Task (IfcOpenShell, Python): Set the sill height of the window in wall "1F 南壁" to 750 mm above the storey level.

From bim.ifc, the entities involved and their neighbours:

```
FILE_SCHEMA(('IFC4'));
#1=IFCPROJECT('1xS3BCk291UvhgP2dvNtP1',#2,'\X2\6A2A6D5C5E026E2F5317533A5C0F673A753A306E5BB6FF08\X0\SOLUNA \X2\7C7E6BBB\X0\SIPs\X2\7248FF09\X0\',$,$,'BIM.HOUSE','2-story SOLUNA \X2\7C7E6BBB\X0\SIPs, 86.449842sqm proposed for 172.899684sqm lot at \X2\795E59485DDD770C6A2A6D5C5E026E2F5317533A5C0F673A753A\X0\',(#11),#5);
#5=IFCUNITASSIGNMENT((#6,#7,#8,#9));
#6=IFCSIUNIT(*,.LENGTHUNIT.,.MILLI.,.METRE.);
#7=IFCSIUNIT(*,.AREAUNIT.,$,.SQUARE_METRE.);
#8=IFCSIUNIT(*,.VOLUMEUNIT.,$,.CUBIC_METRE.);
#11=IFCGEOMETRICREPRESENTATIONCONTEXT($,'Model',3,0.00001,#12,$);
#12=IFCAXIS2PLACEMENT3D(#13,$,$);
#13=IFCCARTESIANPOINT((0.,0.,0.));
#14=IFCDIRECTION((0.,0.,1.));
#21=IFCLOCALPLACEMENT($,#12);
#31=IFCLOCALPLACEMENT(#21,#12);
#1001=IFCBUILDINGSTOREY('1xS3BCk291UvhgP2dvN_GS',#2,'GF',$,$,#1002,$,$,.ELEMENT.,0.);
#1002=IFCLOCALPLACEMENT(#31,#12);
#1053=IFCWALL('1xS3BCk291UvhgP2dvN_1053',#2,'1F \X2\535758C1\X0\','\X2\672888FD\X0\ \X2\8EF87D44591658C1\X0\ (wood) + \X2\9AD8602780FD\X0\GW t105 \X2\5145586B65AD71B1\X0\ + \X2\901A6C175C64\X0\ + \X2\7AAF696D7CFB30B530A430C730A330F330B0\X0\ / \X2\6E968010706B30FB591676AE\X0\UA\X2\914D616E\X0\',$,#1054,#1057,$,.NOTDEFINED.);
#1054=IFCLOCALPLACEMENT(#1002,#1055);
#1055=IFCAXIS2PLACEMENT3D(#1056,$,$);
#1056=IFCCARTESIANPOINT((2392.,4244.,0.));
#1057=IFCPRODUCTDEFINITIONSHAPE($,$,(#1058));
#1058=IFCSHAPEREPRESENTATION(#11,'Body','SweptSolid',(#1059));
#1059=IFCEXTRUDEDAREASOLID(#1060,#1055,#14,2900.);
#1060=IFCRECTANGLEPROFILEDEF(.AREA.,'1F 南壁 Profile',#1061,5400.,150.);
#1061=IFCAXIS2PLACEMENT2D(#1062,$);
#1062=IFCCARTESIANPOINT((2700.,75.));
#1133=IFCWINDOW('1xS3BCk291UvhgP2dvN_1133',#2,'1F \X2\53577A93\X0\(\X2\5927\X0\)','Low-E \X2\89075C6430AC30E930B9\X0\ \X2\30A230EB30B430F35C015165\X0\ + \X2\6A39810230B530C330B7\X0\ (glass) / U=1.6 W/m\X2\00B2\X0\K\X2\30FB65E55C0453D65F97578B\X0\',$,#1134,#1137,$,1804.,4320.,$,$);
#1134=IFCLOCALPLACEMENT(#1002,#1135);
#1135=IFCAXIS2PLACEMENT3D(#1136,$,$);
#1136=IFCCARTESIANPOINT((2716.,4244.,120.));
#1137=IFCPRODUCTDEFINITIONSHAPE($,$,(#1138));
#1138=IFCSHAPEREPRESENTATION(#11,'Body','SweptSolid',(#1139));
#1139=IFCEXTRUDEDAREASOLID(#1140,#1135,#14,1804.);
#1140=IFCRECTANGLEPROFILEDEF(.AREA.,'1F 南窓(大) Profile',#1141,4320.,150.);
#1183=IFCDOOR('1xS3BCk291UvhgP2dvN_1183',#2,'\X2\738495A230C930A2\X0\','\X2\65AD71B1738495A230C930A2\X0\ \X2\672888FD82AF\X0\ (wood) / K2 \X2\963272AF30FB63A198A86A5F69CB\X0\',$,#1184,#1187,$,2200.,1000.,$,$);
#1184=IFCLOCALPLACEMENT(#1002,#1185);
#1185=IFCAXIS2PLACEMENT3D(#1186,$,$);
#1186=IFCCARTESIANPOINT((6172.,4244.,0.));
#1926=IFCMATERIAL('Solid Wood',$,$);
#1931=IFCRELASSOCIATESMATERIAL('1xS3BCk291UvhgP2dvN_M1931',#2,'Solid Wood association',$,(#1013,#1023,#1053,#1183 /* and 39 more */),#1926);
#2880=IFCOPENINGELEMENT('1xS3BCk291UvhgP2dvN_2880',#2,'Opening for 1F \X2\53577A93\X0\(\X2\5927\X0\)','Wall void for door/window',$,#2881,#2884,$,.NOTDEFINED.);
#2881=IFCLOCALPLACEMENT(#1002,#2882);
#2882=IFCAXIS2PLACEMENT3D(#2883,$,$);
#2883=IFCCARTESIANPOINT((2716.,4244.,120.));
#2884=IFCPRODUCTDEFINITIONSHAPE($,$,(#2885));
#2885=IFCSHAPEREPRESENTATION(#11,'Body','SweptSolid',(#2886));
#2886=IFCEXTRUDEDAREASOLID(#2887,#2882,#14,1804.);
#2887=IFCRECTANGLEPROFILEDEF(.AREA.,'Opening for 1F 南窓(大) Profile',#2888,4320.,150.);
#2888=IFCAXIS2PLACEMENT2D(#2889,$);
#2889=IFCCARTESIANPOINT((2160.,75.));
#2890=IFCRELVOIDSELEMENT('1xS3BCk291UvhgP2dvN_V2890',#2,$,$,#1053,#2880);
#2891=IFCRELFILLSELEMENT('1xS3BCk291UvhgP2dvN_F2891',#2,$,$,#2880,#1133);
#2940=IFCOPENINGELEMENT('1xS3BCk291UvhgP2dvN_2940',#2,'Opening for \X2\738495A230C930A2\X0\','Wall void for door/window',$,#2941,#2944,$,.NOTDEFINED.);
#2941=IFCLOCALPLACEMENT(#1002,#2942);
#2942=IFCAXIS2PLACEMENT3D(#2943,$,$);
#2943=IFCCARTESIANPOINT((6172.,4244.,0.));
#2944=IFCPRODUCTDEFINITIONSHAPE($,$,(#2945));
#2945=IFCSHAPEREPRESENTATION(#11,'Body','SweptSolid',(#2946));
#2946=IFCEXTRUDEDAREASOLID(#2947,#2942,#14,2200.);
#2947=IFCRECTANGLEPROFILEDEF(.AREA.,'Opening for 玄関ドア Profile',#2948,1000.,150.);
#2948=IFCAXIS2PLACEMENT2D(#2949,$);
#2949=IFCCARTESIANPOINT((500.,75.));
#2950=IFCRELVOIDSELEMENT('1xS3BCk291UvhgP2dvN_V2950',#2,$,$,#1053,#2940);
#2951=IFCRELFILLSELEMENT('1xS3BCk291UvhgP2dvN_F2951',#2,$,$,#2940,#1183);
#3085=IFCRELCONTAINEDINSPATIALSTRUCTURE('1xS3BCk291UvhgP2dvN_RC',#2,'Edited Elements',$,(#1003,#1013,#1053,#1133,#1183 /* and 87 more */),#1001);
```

```python
import numpy as np
import ifcopenshell
import ifcopenshell.api.geometry
import ifcopenshell.geom
import ifcopenshell.util.element
import ifcopenshell.util.placement
import ifcopenshell.util.shape
import ifcopenshell.util.unit

model = ifcopenshell.open("bim.ifc")
unit_scale = ifcopenshell.util.unit.calculate_unit_scale(model)

window = model.by_guid("1xS3BCk291UvhgP2dvN_1133")
opening = window.FillsVoids[0].RelatingOpeningElement
storey = ifcopenshell.util.element.get_container(window, ifc_class="IfcBuildingStorey")
level = ifcopenshell.util.placement.get_local_placement(storey.ObjectPlacement)[2, 3]

# The opening's origin need not be at the sill, so measure its lowest point.
shape = ifcopenshell.geom.create_shape(ifcopenshell.geom.settings(), opening)
bottom = ifcopenshell.util.shape.get_shape_bottom_elevation(shape, shape.geometry) / unit_scale
dz = level + 750.0 - bottom

shift = np.array([0.0, 0.0, dz])
# The window is not placed relative to its opening, so move both.
for product in (opening, window):
    matrix = ifcopenshell.util.placement.get_local_placement(product.ObjectPlacement)
    matrix[:3, 3] += shift
    ifcopenshell.api.geometry.edit_object_placement(model, product=product, matrix=matrix, is_si=False)

print(f"moved by {dz * unit_scale:+.3f} m")

model.write("bim_updated.ifc")
```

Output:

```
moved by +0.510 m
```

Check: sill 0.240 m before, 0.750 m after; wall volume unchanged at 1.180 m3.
